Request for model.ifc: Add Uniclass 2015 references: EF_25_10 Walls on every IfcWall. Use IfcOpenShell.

First a look at what the model holds.

```python
import ifcopenshell

model = ifcopenshell.open("model.ifc")
print(model.schema)
print("classifications:", [c.Name for c in model.by_type("IfcClassification")])
for ifc_class in ("IfcDoor", "IfcRoof", "IfcStair", "IfcWall", "IfcWindow"):
    print(ifc_class, len(model.by_type(ifc_class)))
```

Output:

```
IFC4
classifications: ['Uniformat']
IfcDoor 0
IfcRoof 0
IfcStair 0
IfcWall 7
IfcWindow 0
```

```python
import ifcopenshell
import ifcopenshell.api.classification

model = ifcopenshell.open("model.ifc")

system = ifcopenshell.api.classification.add_classification(model, classification="Uniclass 2015")

codes = {
    "IfcWall": ("EF_25_10", "Walls"),
}
for ifc_class, (code, name) in codes.items():
    products = model.by_type(ifc_class)
    ifcopenshell.api.classification.add_reference(
        model, products=products, classification=system, identification=code, name=name
    )
    print(code, len(products))

model.write("model_rev.ifc")
```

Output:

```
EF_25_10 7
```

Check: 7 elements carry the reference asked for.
